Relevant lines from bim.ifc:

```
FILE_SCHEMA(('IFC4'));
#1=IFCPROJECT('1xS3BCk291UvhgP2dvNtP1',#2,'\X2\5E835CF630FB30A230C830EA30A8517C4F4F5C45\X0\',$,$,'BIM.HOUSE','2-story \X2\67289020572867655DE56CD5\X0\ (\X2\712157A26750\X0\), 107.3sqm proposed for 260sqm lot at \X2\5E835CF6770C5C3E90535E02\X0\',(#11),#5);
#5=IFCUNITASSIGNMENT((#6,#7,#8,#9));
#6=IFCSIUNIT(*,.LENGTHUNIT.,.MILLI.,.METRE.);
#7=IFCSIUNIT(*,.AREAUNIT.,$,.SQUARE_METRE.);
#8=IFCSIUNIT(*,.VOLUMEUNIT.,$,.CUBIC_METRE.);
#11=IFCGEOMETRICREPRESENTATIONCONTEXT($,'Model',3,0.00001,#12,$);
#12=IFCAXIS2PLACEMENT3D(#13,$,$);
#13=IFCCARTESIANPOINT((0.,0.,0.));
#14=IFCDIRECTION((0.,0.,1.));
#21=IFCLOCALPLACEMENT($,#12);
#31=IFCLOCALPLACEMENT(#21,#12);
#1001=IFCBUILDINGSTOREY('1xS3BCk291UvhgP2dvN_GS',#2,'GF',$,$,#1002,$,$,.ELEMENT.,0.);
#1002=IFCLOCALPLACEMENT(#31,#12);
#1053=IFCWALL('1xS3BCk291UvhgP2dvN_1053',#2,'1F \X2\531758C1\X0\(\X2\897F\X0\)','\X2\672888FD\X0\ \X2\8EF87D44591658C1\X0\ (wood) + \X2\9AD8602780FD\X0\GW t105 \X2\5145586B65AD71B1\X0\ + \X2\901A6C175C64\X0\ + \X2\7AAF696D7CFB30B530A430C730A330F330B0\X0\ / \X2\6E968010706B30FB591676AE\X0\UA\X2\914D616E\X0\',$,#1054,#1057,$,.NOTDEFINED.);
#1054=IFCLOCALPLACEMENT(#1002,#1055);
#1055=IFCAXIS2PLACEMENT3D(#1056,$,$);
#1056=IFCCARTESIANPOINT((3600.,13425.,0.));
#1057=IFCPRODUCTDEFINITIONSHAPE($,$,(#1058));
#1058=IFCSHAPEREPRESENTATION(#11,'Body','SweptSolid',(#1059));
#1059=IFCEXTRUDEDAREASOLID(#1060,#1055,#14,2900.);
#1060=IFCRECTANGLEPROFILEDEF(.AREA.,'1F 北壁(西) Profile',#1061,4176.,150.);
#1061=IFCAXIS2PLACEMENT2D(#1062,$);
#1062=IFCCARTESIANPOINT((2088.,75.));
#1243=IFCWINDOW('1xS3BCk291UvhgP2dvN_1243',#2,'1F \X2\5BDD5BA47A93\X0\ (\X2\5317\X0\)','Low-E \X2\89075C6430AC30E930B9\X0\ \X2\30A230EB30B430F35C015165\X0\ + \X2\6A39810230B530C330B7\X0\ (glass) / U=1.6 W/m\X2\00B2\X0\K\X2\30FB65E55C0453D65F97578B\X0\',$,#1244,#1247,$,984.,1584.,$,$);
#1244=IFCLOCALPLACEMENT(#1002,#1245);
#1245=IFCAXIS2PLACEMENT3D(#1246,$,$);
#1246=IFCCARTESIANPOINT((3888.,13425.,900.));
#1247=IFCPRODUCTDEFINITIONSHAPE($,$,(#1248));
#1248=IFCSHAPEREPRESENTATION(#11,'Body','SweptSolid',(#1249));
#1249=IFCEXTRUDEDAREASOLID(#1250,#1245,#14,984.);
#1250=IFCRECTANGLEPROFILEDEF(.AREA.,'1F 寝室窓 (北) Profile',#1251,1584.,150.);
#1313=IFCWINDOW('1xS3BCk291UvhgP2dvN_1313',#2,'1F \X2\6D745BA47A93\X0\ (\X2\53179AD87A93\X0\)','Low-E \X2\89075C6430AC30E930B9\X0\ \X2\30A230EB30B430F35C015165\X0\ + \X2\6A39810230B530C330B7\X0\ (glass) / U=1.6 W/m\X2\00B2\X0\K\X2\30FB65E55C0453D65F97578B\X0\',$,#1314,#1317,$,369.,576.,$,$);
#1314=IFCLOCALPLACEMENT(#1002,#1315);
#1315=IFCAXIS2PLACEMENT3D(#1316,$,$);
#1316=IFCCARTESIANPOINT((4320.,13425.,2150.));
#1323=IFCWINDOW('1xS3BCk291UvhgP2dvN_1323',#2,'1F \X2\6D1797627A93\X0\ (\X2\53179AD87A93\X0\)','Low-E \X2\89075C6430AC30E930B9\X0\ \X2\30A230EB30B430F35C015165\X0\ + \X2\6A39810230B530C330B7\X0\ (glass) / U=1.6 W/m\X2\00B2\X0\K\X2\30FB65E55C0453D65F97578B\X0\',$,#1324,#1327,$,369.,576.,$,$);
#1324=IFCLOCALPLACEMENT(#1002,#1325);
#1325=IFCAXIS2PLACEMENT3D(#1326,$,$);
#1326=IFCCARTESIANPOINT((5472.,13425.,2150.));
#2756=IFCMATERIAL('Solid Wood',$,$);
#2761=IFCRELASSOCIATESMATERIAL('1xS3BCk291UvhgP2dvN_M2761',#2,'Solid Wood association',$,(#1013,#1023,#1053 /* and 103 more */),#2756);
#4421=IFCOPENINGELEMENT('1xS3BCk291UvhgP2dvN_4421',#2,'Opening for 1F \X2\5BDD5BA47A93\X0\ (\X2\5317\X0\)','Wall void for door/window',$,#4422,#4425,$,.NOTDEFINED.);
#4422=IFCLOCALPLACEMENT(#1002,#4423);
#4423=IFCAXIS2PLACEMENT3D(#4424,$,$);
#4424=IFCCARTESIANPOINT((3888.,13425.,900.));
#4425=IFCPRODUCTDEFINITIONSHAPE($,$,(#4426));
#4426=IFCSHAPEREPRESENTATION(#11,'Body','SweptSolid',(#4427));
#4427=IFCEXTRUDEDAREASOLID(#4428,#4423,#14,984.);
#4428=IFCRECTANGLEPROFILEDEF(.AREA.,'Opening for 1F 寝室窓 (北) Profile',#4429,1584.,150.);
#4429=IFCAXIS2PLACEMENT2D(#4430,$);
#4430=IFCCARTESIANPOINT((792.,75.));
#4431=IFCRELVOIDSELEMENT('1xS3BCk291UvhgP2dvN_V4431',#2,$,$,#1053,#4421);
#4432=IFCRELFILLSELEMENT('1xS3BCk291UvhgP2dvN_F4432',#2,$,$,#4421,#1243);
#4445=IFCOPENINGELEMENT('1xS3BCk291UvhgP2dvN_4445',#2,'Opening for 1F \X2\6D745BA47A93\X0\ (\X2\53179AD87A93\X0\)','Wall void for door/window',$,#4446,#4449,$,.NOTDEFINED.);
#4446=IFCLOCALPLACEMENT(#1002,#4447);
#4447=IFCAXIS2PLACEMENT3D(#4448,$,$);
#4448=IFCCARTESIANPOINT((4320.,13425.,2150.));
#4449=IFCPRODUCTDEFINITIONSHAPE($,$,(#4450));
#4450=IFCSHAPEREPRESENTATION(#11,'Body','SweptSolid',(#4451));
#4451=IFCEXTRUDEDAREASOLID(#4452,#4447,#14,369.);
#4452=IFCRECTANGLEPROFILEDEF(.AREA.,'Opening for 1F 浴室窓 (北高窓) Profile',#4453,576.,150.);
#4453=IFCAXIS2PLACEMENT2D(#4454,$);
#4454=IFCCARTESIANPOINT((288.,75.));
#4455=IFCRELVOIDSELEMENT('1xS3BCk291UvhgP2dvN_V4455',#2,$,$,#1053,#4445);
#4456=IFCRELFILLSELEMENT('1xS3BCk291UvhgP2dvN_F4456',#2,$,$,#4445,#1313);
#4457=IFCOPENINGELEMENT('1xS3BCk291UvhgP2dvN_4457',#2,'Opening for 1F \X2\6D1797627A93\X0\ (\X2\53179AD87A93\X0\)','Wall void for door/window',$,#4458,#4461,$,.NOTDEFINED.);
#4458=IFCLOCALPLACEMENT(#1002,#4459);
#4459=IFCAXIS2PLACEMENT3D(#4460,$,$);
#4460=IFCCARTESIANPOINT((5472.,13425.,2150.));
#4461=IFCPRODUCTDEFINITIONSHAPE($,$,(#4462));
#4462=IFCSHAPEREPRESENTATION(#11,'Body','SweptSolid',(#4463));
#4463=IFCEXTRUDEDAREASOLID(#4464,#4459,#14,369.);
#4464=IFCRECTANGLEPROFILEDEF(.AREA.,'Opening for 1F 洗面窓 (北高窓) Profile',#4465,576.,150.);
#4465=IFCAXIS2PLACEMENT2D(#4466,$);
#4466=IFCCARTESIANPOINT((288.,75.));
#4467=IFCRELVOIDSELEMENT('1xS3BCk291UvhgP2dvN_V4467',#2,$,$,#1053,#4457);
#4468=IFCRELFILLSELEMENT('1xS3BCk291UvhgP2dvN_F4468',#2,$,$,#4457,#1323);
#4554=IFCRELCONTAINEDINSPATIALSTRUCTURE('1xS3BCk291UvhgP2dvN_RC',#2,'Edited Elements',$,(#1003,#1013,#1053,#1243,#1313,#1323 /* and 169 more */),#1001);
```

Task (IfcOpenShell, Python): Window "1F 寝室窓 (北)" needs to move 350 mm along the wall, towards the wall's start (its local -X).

```python
import ifcopenshell
import ifcopenshell.api.geometry
import ifcopenshell.util.placement

model = ifcopenshell.open("bim.ifc")

window = model.by_id(1243)
opening = window.FillsVoids[0].RelatingOpeningElement
wall = opening.VoidsElements[0].RelatingBuildingElement

wall_matrix = ifcopenshell.util.placement.get_local_placement(wall.ObjectPlacement)
shift = wall_matrix[:3, 0] * -350.0
before = ifcopenshell.util.placement.get_local_placement(window.ObjectPlacement)[:3, 3].copy()

# The window is not placed relative to its opening, so move both.
for product in (opening, window):
    matrix = ifcopenshell.util.placement.get_local_placement(product.ObjectPlacement)
    matrix[:3, 3] += shift
    ifcopenshell.api.geometry.edit_object_placement(model, product=product, matrix=matrix, is_si=False)

after = ifcopenshell.util.placement.get_local_placement(window.ObjectPlacement)[:3, 3]
print("window moved by", (after - before).round(3) + 0.0)

model.write("bim_v2.ifc")
```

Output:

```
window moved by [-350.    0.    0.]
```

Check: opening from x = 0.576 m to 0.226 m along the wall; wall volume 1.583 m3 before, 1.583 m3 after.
